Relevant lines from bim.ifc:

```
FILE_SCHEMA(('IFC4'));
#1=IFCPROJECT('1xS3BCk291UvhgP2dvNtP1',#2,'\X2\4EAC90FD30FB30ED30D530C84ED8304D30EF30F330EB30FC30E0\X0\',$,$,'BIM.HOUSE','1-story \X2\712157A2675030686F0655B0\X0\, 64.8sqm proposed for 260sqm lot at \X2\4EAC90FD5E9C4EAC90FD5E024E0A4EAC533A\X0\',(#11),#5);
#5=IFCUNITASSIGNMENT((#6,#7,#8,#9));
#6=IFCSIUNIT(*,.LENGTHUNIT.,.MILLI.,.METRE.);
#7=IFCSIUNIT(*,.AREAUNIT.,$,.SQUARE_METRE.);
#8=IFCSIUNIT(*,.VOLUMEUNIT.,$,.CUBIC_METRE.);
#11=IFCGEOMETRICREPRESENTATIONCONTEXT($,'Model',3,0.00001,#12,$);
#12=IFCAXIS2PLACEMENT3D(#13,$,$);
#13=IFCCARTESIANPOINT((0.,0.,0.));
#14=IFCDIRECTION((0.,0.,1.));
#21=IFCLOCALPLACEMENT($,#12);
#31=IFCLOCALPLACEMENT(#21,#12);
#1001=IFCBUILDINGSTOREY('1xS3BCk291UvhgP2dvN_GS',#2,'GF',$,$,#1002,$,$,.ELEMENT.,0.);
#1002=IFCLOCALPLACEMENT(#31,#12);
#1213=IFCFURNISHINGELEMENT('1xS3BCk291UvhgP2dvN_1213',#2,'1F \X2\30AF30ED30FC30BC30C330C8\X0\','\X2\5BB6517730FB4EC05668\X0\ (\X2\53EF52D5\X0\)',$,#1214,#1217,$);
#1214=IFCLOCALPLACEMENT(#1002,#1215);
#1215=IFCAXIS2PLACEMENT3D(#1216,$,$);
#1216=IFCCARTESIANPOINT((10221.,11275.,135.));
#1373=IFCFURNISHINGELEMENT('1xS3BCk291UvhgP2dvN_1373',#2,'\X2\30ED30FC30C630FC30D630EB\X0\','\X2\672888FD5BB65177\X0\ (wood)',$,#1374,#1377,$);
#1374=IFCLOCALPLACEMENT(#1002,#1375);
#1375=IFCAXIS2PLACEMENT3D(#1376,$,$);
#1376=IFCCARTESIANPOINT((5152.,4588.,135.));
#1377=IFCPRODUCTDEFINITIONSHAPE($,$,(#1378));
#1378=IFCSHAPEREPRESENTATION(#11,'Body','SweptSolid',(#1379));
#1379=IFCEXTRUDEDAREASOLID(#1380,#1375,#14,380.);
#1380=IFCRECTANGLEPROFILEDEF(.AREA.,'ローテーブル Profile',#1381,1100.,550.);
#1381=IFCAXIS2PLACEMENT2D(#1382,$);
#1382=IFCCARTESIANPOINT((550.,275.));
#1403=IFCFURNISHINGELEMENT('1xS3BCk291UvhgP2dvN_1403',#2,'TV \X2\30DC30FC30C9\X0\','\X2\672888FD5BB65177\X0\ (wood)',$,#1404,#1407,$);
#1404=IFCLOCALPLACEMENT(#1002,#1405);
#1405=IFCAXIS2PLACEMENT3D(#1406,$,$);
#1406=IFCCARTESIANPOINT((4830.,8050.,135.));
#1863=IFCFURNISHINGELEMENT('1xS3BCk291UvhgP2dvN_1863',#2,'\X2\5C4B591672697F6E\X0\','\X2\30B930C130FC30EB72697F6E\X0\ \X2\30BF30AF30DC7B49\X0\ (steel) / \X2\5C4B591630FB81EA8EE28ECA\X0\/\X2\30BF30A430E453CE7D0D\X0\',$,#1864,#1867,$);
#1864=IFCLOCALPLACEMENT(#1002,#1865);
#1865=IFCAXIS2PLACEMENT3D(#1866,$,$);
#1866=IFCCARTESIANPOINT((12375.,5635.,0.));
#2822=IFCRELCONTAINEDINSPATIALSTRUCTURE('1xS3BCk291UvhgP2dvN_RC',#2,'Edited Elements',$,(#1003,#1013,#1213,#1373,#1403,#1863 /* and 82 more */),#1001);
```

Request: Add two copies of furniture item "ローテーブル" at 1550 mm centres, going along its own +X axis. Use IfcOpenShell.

```python
import ifcopenshell
import ifcopenshell.api.geometry
import ifcopenshell.api.root
import ifcopenshell.util.element
import ifcopenshell.util.placement
import ifcopenshell.util.unit

model = ifcopenshell.open("bim.ifc")
unit_scale = ifcopenshell.util.unit.calculate_unit_scale(model)


def reuse_history(source, copy):
    """copy_class also copies each property set's owner history, people and application; keep the originals."""
    for rel in copy.IsDefinedBy:
        if rel.is_a("IfcRelDefinesByProperties") and (history := rel.RelatingPropertyDefinition.OwnerHistory):
            rel.RelatingPropertyDefinition.OwnerHistory = source.OwnerHistory
            ifcopenshell.util.element.remove_deep2(model, history)


source = model.by_id(1373)
base = ifcopenshell.util.placement.get_local_placement(source.ObjectPlacement)
step = base[:3, 0] * 1.55 / unit_scale

for i in range(1, 3):
    copy = ifcopenshell.api.root.copy_class(model, product=source)
    copy.Representation = ifcopenshell.util.element.copy_deep(
        model, source.Representation, exclude=["IfcGeometricRepresentationContext", "IfcRepresentationMap"]
    )
    reuse_history(source, copy)
    matrix = base.copy()
    matrix[:3, 3] += i * step
    print("added at", matrix[:3, 3].round(3) + 0.0)
    ifcopenshell.api.geometry.edit_object_placement(model, product=copy, matrix=matrix, is_si=False)

model.write("bim_updated.ifc")
```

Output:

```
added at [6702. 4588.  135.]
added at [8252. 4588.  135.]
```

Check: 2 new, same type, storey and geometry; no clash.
